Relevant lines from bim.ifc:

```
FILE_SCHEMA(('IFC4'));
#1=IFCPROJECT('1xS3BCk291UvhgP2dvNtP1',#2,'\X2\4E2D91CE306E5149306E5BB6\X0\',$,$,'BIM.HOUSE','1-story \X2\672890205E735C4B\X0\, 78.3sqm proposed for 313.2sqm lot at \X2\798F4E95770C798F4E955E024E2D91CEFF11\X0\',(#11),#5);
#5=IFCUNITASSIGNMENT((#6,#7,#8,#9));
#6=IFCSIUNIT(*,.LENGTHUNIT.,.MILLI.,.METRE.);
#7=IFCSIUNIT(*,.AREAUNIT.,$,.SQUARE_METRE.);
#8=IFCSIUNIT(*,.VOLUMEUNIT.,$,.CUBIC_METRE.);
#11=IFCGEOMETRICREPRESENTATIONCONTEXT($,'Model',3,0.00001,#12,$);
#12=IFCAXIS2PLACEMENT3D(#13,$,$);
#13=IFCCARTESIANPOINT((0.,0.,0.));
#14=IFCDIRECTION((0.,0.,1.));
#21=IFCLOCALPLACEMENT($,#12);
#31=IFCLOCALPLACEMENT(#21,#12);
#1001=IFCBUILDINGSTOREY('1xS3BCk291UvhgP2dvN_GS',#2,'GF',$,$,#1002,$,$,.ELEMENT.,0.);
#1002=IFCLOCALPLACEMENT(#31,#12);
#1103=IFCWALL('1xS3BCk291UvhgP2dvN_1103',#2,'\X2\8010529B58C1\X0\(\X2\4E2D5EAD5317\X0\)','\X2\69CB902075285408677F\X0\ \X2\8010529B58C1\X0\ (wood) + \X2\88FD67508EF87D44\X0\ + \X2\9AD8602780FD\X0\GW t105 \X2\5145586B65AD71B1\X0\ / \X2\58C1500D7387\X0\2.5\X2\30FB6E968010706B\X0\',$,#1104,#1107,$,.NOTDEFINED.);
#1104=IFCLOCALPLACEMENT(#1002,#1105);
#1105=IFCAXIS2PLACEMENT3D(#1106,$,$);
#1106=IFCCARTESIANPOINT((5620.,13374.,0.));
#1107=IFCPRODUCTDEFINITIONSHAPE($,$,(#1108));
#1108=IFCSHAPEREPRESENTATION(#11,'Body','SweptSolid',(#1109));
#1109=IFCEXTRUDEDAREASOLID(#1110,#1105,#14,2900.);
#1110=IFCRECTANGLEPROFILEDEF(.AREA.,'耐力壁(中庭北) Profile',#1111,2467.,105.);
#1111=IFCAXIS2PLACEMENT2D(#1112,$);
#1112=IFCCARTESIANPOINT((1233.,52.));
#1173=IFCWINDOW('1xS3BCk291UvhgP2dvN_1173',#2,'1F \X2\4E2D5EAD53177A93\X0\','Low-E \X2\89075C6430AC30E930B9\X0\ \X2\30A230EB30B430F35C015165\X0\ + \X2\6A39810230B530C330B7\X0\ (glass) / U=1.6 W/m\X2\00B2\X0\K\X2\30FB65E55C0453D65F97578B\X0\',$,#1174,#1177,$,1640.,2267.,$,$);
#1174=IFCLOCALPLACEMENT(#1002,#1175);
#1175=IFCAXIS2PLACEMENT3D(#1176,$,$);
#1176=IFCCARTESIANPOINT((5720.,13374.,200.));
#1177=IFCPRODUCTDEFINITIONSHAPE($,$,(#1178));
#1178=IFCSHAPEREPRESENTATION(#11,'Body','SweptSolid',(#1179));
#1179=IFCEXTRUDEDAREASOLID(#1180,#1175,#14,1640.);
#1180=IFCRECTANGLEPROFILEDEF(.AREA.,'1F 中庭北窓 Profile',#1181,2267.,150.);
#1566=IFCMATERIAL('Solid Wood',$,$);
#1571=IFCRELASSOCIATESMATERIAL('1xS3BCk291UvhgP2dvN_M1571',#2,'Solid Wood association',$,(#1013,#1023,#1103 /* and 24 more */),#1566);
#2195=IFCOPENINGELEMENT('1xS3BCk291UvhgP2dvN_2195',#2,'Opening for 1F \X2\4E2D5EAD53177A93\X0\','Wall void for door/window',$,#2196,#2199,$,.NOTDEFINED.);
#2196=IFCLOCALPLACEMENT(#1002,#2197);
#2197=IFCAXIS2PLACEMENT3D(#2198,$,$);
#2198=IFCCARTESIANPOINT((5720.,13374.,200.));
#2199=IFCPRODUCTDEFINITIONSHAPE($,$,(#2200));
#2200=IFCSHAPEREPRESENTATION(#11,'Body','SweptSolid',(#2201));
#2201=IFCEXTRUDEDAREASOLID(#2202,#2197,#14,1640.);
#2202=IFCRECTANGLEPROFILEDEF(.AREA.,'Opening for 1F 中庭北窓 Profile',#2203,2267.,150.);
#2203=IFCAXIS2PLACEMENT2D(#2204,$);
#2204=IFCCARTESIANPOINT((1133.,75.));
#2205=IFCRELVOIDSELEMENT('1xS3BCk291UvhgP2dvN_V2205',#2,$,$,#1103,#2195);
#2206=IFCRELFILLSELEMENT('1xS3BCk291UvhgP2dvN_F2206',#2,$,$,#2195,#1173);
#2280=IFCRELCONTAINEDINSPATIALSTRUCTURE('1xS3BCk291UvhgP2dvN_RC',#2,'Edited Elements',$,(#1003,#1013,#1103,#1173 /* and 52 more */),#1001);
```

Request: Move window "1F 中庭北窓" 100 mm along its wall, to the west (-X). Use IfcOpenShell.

```python
import ifcopenshell
import ifcopenshell.api.geometry
import ifcopenshell.util.placement

model = ifcopenshell.open("bim.ifc")

window = model.by_guid("1xS3BCk291UvhgP2dvN_1173")
opening = window.FillsVoids[0].RelatingOpeningElement
wall = opening.VoidsElements[0].RelatingBuildingElement

wall_matrix = ifcopenshell.util.placement.get_local_placement(wall.ObjectPlacement)
shift = wall_matrix[:3, 0] * -100.0
before = ifcopenshell.util.placement.get_local_placement(window.ObjectPlacement)[:3, 3].copy()

# The window is not placed relative to its opening, so move both.
for product in (opening, window):
    matrix = ifcopenshell.util.placement.get_local_placement(product.ObjectPlacement)
    matrix[:3, 3] += shift
    ifcopenshell.api.geometry.edit_object_placement(model, product=product, matrix=matrix, is_si=False)

after = ifcopenshell.util.placement.get_local_placement(window.ObjectPlacement)[:3, 3]
print("window moved by", (after - before).round(3) + 0.0)

model.write("bim_rev.ifc")
```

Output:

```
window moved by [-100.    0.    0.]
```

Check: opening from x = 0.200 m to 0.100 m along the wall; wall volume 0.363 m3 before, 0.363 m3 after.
